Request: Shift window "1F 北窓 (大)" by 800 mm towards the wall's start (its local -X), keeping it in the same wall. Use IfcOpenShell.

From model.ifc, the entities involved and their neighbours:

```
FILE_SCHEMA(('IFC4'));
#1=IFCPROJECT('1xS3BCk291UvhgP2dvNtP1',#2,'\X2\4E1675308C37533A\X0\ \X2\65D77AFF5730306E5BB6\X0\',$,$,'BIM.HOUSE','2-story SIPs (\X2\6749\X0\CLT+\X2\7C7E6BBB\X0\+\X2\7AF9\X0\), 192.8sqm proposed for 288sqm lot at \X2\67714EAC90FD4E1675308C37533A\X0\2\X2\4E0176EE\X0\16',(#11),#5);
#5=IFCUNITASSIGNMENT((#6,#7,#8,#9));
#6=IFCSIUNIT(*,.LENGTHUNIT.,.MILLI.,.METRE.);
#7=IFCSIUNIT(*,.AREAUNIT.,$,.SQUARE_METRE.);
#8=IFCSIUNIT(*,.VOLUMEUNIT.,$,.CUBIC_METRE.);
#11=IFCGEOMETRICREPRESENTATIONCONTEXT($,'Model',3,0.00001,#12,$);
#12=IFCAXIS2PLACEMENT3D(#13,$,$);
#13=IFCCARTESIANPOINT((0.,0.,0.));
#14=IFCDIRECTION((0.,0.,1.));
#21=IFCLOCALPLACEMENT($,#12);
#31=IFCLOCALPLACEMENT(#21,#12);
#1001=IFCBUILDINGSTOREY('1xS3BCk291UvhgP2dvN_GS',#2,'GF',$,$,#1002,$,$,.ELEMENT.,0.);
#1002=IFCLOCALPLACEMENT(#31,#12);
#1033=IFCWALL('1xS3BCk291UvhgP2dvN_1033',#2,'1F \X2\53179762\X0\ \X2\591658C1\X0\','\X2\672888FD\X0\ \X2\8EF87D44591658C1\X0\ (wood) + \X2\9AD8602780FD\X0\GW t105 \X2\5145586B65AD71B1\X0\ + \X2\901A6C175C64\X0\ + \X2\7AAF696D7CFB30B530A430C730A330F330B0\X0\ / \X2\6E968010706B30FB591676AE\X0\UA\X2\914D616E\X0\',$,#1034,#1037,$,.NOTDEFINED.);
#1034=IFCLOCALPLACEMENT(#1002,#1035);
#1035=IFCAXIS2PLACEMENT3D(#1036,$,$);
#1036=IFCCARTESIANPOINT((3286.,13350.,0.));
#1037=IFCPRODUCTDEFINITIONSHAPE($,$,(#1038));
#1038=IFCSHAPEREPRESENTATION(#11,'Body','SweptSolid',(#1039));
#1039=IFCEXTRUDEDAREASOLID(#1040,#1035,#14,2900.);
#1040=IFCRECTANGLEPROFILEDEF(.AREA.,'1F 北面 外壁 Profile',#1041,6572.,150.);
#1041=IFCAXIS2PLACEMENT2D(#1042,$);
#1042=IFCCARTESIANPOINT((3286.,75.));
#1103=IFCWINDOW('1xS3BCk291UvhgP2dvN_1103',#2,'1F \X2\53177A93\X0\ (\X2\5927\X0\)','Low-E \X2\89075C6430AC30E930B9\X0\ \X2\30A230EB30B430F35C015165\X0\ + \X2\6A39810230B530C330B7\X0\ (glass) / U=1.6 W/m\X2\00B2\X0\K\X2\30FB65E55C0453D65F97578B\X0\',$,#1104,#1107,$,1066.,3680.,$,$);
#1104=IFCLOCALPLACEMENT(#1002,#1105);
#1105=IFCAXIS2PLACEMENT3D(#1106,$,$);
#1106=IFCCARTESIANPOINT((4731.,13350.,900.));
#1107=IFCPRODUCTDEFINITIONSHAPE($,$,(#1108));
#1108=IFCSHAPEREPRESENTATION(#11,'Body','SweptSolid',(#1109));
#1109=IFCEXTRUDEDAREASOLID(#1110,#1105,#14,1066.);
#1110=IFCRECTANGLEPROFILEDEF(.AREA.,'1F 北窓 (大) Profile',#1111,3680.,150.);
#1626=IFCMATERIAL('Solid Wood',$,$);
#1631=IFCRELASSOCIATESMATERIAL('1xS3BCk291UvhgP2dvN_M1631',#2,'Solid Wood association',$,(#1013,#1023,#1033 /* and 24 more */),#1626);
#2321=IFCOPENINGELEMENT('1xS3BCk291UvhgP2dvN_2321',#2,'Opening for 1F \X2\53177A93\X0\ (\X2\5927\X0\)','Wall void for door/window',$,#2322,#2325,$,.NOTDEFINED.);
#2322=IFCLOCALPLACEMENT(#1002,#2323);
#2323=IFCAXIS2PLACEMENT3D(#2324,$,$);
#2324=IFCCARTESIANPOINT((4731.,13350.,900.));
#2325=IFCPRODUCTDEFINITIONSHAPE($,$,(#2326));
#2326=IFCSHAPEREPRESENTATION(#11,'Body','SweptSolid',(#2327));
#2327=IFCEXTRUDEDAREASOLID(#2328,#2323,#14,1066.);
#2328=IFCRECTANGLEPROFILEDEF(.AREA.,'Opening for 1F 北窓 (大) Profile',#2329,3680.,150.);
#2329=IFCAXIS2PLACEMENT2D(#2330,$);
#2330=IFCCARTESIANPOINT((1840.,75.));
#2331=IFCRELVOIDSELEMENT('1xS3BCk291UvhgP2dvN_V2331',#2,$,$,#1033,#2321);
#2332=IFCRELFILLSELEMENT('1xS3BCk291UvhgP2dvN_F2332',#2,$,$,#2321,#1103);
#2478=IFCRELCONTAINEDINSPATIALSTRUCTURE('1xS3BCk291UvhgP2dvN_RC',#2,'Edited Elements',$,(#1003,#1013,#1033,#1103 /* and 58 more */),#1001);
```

```python
import ifcopenshell
import ifcopenshell.api.geometry
import ifcopenshell.util.placement

model = ifcopenshell.open("model.ifc")

window = model.by_guid("1xS3BCk291UvhgP2dvN_1103")
opening = window.FillsVoids[0].RelatingOpeningElement
wall = opening.VoidsElements[0].RelatingBuildingElement

wall_matrix = ifcopenshell.util.placement.get_local_placement(wall.ObjectPlacement)
shift = wall_matrix[:3, 0] * -800.0
before = ifcopenshell.util.placement.get_local_placement(window.ObjectPlacement)[:3, 3].copy()

# The window is not placed relative to its opening, so move both.
for product in (opening, window):
    matrix = ifcopenshell.util.placement.get_local_placement(product.ObjectPlacement)
    matrix[:3, 3] += shift
    ifcopenshell.api.geometry.edit_object_placement(model, product=product, matrix=matrix, is_si=False)

after = ifcopenshell.util.placement.get_local_placement(window.ObjectPlacement)[:3, 3]
print("window moved by", (after - before).round(3) + 0.0)

model.write("model_updated.ifc")
```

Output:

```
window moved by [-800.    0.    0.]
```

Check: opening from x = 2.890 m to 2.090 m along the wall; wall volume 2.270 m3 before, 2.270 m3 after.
